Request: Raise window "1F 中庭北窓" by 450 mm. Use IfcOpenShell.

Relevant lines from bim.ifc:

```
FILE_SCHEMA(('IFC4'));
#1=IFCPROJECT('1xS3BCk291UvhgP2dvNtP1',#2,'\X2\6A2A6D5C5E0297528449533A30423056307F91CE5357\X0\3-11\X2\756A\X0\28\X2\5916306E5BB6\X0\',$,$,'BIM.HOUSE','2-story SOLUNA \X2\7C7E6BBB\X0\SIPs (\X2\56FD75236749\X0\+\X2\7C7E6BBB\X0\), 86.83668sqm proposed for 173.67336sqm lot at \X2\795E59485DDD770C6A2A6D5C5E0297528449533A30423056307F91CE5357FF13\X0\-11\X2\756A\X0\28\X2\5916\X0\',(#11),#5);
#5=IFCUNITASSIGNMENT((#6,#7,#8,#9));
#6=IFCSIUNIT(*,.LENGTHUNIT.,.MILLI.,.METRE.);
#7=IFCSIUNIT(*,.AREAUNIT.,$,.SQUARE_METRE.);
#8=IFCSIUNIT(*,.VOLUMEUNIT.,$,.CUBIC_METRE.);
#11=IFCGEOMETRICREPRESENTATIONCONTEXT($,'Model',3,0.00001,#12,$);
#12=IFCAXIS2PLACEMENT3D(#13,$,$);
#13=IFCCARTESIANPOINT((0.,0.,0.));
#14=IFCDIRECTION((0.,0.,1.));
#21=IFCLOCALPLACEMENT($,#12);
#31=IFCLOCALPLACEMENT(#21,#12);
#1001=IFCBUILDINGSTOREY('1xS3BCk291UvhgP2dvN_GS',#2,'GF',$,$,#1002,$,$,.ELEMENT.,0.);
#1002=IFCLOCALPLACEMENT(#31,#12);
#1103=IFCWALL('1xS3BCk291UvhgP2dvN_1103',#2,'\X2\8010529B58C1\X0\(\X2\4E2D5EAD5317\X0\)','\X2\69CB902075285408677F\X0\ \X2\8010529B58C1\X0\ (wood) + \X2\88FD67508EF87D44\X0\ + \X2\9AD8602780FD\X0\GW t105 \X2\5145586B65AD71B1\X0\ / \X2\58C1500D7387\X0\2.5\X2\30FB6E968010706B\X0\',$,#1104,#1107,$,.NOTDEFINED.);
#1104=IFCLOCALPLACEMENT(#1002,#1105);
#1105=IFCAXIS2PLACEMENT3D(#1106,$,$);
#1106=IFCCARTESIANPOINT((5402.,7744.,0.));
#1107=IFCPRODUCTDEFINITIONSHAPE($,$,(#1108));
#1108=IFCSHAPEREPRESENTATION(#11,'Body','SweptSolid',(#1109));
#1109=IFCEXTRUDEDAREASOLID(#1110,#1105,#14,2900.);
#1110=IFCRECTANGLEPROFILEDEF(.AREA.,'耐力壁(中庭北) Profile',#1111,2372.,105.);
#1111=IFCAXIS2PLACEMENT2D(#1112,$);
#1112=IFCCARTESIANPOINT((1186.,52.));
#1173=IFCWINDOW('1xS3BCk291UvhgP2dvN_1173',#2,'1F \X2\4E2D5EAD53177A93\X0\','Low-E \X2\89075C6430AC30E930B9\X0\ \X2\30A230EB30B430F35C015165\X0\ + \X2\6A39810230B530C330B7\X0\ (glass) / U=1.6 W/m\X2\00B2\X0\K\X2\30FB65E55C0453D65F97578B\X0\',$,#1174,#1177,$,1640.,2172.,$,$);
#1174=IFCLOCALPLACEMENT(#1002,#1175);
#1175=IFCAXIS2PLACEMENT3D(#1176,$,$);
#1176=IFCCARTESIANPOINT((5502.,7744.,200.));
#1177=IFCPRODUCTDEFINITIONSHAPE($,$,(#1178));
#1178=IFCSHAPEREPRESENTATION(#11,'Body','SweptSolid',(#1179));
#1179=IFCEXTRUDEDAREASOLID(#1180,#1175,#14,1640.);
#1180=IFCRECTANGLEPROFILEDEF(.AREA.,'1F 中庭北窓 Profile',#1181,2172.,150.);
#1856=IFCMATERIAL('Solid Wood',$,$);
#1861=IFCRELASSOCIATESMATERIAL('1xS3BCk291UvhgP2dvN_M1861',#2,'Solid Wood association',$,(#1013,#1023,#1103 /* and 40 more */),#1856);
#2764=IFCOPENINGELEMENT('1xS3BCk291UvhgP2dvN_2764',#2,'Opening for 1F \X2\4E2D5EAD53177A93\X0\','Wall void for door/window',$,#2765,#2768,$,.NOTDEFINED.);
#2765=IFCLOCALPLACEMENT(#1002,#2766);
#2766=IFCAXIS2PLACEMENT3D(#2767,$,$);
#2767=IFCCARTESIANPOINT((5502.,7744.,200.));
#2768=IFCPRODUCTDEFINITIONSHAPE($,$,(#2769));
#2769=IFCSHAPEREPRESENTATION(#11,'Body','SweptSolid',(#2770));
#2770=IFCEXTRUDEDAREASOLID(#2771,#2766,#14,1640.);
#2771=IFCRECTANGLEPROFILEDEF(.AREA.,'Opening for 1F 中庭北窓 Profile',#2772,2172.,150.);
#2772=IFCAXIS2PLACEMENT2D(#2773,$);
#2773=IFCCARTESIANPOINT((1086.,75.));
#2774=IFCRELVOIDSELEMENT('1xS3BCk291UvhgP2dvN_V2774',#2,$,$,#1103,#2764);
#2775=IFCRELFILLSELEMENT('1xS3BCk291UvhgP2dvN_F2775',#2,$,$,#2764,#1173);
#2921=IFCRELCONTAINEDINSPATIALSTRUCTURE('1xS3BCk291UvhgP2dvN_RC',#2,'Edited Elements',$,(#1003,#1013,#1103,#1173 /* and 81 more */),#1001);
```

```python
import numpy as np
import ifcopenshell
import ifcopenshell.api.geometry
import ifcopenshell.util.placement
import ifcopenshell.util.unit

model = ifcopenshell.open("bim.ifc")
unit_scale = ifcopenshell.util.unit.calculate_unit_scale(model)

window = model.by_guid("1xS3BCk291UvhgP2dvN_1173")
opening = window.FillsVoids[0].RelatingOpeningElement
dz = 0.45 / unit_scale

shift = np.array([0.0, 0.0, dz])
# The window is not placed relative to its opening, so move both.
for product in (opening, window):
    matrix = ifcopenshell.util.placement.get_local_placement(product.ObjectPlacement)
    matrix[:3, 3] += shift
    ifcopenshell.api.geometry.edit_object_placement(model, product=product, matrix=matrix, is_si=False)

print(f"moved by {dz * unit_scale:+.3f} m")

model.write("bim-out.ifc")
```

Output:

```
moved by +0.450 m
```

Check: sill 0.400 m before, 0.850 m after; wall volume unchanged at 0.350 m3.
